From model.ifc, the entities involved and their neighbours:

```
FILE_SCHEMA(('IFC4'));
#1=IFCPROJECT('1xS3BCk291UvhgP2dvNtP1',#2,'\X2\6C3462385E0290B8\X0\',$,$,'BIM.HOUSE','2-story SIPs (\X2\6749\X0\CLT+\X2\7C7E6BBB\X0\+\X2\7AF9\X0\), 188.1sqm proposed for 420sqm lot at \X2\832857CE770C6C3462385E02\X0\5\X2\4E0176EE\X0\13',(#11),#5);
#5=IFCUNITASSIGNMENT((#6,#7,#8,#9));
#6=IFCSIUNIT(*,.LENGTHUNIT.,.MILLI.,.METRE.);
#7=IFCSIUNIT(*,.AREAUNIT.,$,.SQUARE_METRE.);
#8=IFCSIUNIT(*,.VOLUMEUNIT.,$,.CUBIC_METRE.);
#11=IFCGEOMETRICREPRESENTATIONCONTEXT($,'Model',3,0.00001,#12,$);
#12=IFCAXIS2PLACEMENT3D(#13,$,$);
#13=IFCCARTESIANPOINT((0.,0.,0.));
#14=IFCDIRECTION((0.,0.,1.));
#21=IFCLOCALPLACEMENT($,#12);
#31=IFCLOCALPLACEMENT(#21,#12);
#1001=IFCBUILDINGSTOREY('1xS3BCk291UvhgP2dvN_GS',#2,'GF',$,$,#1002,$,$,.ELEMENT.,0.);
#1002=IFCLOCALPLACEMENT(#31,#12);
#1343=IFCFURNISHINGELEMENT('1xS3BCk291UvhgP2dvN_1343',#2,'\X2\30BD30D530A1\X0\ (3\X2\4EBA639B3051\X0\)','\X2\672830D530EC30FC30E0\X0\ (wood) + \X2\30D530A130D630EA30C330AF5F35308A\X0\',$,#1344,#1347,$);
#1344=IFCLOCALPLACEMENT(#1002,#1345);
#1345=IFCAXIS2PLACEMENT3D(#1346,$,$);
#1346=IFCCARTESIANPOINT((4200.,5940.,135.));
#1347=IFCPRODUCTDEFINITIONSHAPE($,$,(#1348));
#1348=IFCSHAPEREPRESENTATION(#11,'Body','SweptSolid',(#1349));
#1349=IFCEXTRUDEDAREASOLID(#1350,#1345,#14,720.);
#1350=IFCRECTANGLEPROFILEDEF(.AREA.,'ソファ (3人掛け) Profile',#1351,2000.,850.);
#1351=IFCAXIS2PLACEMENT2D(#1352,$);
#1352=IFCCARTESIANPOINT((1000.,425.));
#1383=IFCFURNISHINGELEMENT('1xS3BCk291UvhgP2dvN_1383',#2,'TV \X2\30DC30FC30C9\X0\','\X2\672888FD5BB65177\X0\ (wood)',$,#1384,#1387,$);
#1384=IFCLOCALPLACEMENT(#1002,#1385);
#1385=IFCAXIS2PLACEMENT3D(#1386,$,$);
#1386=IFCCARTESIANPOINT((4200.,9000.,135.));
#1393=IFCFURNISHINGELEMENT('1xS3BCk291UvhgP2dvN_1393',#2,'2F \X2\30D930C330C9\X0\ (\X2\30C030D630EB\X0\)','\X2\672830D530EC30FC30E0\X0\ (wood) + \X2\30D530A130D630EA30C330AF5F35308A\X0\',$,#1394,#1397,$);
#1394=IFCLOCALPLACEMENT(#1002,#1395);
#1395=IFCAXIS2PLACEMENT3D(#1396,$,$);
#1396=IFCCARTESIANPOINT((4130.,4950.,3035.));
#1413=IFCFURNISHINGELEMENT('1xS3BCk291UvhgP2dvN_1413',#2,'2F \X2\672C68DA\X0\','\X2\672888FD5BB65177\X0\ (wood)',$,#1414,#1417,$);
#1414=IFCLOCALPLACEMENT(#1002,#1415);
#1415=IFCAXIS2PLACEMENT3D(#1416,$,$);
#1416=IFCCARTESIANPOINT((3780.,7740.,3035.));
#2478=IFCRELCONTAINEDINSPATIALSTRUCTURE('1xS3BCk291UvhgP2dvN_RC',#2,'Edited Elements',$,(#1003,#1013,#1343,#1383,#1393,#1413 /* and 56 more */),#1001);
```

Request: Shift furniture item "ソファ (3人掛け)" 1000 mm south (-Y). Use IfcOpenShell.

```python
import ifcopenshell
import ifcopenshell.api.geometry
import ifcopenshell.util.placement
import ifcopenshell.util.unit

model = ifcopenshell.open("model.ifc")
unit_scale = ifcopenshell.util.unit.calculate_unit_scale(model)

item = model.by_guid("1xS3BCk291UvhgP2dvN_1343")
matrix = ifcopenshell.util.placement.get_local_placement(item.ObjectPlacement)
matrix[1, 3] -= 1 / unit_scale
ifcopenshell.api.geometry.edit_object_placement(model, product=item, matrix=matrix, is_si=False)

print(ifcopenshell.util.placement.get_local_placement(item.ObjectPlacement).round(3) + 0.0)

model.write("model_rev.ifc")
```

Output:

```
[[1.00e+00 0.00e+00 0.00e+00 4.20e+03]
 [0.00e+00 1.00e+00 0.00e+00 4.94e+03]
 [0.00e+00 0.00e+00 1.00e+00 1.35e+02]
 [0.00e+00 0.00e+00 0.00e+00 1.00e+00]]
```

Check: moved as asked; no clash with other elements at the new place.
